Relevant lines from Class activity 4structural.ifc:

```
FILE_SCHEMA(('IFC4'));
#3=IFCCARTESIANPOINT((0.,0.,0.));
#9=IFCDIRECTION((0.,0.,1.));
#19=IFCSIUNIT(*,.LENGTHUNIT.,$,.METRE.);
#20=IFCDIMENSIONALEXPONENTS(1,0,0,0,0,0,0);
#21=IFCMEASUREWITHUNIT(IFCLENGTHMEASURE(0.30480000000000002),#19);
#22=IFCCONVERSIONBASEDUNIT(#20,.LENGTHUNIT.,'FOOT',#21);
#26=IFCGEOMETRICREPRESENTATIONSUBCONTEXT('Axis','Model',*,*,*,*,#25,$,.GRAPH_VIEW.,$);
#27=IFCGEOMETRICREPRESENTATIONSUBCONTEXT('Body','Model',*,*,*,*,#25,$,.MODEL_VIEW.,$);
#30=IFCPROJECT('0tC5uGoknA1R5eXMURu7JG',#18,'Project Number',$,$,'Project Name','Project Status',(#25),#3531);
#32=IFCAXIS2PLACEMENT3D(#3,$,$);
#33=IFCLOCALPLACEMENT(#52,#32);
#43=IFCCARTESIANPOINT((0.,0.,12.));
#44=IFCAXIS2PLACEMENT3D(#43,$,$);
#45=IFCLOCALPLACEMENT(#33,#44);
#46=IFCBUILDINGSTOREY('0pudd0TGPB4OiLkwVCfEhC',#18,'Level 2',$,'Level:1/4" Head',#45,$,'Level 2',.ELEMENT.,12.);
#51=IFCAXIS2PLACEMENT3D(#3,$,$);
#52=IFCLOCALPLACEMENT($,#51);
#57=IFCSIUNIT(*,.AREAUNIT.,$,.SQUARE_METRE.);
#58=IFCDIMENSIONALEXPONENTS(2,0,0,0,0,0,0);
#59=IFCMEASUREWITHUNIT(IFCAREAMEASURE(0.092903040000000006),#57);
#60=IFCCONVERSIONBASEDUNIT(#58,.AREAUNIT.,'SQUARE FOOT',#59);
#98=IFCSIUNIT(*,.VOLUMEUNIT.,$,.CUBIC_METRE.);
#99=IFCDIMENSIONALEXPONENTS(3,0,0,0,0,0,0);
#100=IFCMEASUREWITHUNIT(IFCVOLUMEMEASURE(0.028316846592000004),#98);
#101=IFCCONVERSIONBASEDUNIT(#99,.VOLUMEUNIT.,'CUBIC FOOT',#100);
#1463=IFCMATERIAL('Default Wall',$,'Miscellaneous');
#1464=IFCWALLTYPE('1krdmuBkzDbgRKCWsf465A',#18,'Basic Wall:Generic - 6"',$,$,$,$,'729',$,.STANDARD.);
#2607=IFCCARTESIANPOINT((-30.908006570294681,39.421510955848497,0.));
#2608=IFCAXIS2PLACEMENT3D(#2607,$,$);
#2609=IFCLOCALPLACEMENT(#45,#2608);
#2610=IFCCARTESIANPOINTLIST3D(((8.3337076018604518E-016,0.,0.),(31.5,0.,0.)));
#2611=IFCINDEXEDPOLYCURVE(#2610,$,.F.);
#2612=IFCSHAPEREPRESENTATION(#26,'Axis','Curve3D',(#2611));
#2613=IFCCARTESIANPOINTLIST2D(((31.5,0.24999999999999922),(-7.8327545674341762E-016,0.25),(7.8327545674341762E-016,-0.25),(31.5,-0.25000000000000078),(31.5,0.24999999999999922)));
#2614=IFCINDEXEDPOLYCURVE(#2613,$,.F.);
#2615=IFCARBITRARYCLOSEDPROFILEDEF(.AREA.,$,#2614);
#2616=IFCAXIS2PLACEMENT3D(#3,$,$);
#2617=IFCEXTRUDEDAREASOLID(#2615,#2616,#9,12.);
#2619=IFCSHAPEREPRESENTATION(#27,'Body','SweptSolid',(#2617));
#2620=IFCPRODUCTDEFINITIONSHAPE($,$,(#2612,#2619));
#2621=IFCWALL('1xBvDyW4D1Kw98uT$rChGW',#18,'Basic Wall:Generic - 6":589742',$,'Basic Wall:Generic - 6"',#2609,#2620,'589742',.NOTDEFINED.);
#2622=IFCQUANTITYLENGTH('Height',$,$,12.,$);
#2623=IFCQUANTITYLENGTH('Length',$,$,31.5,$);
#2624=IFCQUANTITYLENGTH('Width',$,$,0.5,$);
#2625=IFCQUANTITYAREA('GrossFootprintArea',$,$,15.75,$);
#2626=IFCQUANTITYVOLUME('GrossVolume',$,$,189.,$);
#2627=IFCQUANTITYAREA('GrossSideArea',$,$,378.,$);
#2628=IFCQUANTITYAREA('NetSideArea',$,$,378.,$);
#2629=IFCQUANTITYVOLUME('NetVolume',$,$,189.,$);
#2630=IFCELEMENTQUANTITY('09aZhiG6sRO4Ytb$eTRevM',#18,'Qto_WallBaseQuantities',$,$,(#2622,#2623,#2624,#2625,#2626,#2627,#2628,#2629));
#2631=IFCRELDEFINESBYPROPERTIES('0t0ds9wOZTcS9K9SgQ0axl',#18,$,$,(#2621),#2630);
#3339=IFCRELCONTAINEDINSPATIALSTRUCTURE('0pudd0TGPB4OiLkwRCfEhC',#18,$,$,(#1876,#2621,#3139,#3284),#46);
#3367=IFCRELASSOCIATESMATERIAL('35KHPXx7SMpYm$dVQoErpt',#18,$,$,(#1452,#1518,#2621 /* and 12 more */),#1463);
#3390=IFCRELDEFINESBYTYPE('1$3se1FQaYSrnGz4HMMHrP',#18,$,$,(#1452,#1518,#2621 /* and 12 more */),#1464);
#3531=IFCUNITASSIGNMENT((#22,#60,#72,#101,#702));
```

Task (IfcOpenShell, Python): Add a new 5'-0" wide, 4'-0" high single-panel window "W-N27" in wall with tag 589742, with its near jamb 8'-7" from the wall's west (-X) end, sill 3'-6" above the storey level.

```python
import numpy as np
import ifcopenshell
import ifcopenshell.api.feature
import ifcopenshell.api.geometry
import ifcopenshell.api.pset
import ifcopenshell.api.root
import ifcopenshell.api.spatial
import ifcopenshell.geom
import ifcopenshell.util.element
import ifcopenshell.util.placement
import ifcopenshell.util.representation
import ifcopenshell.util.shape
import ifcopenshell.util.unit

model = ifcopenshell.open("Class activity 4structural.ifc")
unit_scale = ifcopenshell.util.unit.calculate_unit_scale(model)
area_scale = ifcopenshell.util.unit.calculate_unit_scale(model, "AREAUNIT")
volume_scale = ifcopenshell.util.unit.calculate_unit_scale(model, "VOLUMEUNIT")
settings = ifcopenshell.geom.settings()


def volume(element):
    """Net volume in cubic metres, openings subtracted."""
    shape = ifcopenshell.geom.create_shape(settings, element)
    return ifcopenshell.util.shape.get_volume(shape.geometry)


wall = model.by_guid("1xBvDyW4D1Kw98uT$rChGW")
storey = ifcopenshell.util.element.get_container(wall, ifc_class="IfcBuildingStorey")
context = ifcopenshell.util.representation.get_context(model, "Model", "Body", "MODEL_VIEW")
before = volume(wall)

width, height, from_end, sill = 1.524, 1.2192, 2.6162, 1.0668  # metres

# The wall runs along its own X axis, and the end named is its -X end.
wall_shape = ifcopenshell.geom.create_shape(settings, wall)
x, y, z = ifcopenshell.util.shape.get_vertices(wall_shape.geometry).T
start = x.min() + from_end
face, thickness = float(y.min()), float(y.max() - y.min())
wall_matrix = ifcopenshell.util.placement.get_local_placement(wall.ObjectPlacement)
level = ifcopenshell.util.placement.get_local_placement(storey.ObjectPlacement)[2, 3]


def in_wall(x, y):
    """Placement at x, y metres in the wall's axes, at sill height."""
    matrix = wall_matrix.copy()
    matrix[:, 3] = wall_matrix @ np.array([x / unit_scale, y / unit_scale, 0.0, 1.0])
    matrix[2, 3] = level + sill / unit_scale
    return matrix


# Opening: a box that overshoots both wall faces by 50 mm.
opening = ifcopenshell.api.root.create_entity(model, ifc_class="IfcOpeningElement", predefined_type="OPENING")
box = ifcopenshell.api.geometry.add_wall_representation(
    model, context=context, length=width, height=height, thickness=thickness + 0.1
)
ifcopenshell.api.geometry.assign_representation(model, product=opening, representation=box)
ifcopenshell.api.geometry.edit_object_placement(model, product=opening, matrix=in_wall(start, face - 0.05), is_si=False)
ifcopenshell.api.feature.add_feature(model, feature=opening, element=wall)

window = ifcopenshell.api.root.create_entity(model, ifc_class="IfcWindow", name="W-N27", predefined_type="WINDOW")
window.OverallWidth, window.OverallHeight = width / unit_scale, height / unit_scale
window.PartitioningType = "SINGLE_PANEL"
body = ifcopenshell.api.geometry.add_window_representation(
    model,
    context=context,
    overall_width=window.OverallWidth,
    overall_height=window.OverallHeight,
    partition_type="SINGLE_PANEL",
)
ifcopenshell.api.geometry.assign_representation(model, product=window, representation=body)
ifcopenshell.api.spatial.assign_container(model, products=[window], relating_structure=storey)
ifcopenshell.api.feature.add_filling(model, opening=opening, element=window)

# Centre the window in the wall's thickness.
ifcopenshell.api.geometry.edit_object_placement(model, product=window, matrix=in_wall(start, face), is_si=False)
window_shape = ifcopenshell.geom.create_shape(settings, window)
depth = ifcopenshell.util.shape.get_vertices(window_shape.geometry)[:, 1]
offset = face + thickness / 2 - (depth.min() + depth.max()) / 2
ifcopenshell.api.geometry.edit_object_placement(model, product=window, matrix=in_wall(start, offset), is_si=False)

after = volume(wall)

# Update the wall's stored quantities.
qto = model.by_id(ifcopenshell.util.element.get_pset(wall, "Qto_WallBaseQuantities", should_inherit=False)["id"])
ifcopenshell.api.pset.edit_qto(model, qto=qto, properties={
    "NetSideArea": after / thickness / area_scale,
    "NetVolume": after / volume_scale,
})

print(f"wall volume {before:.3f} -> {after:.3f} m3")

model.write("Class activity 4structural_updated.ifc")
```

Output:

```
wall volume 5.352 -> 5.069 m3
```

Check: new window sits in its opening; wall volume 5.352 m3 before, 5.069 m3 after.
